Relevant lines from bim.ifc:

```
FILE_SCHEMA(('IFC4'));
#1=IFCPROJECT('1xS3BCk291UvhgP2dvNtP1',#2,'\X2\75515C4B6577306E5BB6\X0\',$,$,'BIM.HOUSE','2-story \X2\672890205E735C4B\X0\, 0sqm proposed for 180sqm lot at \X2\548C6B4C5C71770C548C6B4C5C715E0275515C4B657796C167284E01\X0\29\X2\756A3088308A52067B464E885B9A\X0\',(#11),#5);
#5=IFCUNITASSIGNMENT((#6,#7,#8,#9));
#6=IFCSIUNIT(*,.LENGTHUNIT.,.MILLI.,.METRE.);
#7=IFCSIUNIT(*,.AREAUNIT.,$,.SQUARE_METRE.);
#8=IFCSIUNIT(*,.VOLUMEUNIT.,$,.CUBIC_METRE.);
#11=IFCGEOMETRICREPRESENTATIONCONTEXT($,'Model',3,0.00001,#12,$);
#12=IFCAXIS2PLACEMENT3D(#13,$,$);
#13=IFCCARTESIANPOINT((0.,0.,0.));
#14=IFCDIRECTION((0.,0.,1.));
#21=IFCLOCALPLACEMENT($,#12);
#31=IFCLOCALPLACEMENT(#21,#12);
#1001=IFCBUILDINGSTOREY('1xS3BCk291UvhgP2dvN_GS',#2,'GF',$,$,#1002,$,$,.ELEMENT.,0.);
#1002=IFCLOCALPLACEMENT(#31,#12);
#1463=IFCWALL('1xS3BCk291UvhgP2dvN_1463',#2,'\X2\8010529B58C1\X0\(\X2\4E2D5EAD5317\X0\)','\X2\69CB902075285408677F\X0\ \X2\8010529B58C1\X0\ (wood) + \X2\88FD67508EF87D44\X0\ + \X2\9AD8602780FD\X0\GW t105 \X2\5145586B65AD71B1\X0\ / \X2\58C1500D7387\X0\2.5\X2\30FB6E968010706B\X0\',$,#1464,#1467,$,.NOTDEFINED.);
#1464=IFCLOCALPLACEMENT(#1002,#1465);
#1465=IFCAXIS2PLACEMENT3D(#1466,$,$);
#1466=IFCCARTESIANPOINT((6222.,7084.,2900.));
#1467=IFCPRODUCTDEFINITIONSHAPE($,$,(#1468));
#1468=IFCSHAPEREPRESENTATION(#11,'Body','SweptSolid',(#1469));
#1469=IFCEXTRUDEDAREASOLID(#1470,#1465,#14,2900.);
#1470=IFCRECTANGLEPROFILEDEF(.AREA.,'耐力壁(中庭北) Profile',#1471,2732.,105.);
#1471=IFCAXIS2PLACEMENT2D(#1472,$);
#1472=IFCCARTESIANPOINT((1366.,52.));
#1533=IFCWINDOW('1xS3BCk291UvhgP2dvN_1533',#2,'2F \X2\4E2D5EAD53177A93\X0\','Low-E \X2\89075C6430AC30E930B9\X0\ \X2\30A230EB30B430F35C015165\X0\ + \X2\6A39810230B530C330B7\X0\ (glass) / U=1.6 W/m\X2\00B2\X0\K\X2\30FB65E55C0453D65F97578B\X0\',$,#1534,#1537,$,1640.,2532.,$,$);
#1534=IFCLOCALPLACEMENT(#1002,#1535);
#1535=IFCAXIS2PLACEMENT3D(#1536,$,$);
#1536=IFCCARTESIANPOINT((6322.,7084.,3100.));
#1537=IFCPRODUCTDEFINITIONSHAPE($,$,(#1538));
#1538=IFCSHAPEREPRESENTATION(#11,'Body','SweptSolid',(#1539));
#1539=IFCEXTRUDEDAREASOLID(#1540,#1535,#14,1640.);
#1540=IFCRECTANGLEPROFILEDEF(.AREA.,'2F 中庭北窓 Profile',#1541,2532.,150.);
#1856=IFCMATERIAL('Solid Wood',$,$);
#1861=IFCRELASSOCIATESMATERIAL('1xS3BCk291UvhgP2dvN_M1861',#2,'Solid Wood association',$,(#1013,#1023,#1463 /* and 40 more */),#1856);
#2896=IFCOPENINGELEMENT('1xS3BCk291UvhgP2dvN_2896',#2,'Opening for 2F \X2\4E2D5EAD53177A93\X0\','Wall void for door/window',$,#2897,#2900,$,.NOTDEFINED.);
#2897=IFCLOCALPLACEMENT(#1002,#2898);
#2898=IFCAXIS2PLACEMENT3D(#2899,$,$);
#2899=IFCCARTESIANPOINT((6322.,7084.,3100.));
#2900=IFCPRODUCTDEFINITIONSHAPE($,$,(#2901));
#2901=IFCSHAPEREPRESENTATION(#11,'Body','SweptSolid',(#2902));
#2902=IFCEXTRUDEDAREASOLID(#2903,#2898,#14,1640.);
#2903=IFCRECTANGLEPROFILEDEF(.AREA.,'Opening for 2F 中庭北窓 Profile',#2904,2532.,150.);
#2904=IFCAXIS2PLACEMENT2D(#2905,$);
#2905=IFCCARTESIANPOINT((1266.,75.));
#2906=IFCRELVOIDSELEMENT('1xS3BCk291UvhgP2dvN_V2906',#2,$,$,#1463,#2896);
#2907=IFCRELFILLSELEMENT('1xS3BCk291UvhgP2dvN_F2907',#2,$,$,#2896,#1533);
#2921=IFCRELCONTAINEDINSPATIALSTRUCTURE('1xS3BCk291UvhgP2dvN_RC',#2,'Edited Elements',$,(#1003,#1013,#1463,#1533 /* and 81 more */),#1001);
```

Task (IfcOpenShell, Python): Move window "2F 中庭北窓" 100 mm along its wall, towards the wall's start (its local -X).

```python
import ifcopenshell
import ifcopenshell.api.geometry
import ifcopenshell.util.placement
import ifcopenshell.util.unit

model = ifcopenshell.open("bim.ifc")
unit_scale = ifcopenshell.util.unit.calculate_unit_scale(model)

window = model.by_id(1533)
opening = window.FillsVoids[0].RelatingOpeningElement
wall = opening.VoidsElements[0].RelatingBuildingElement

wall_matrix = ifcopenshell.util.placement.get_local_placement(wall.ObjectPlacement)
shift = wall_matrix[:3, 0] * -0.1 / unit_scale
before = ifcopenshell.util.placement.get_local_placement(window.ObjectPlacement)[:3, 3].copy()

# The window is not placed relative to its opening, so move both.
for product in (opening, window):
    matrix = ifcopenshell.util.placement.get_local_placement(product.ObjectPlacement)
    matrix[:3, 3] += shift
    ifcopenshell.api.geometry.edit_object_placement(model, product=product, matrix=matrix, is_si=False)

after = ifcopenshell.util.placement.get_local_placement(window.ObjectPlacement)[:3, 3]
print("window moved by", (after - before).round(3) + 0.0)

model.write("bim-out.ifc")
```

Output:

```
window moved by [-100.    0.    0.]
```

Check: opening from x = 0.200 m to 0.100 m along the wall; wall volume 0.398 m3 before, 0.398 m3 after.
